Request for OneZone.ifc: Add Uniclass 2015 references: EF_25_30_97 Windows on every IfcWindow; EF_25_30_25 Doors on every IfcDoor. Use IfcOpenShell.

First a look at what the model holds.

```python
import ifcopenshell

model = ifcopenshell.open("OneZone.ifc")
print(model.schema)
print("classifications:", [c.Name for c in model.by_type("IfcClassification")])
for ifc_class in ("IfcDoor", "IfcRoof", "IfcStair", "IfcWall", "IfcWindow"):
    print(ifc_class, len(model.by_type(ifc_class)))
```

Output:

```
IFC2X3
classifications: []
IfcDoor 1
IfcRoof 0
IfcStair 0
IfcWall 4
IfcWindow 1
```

```python
import ifcopenshell
import ifcopenshell.api.classification

model = ifcopenshell.open("OneZone.ifc")

# IFC2X3 requires Source and Edition and has no link from the project to the system.
system = model.create_entity("IfcClassification", Source="NBS", Edition="2015", Name="Uniclass 2015")

codes = {
    "IfcWindow": ("EF_25_30_97", "Windows"),
    "IfcDoor": ("EF_25_30_25", "Doors"),
}
for ifc_class, (code, name) in codes.items():
    products = model.by_type(ifc_class)
    ifcopenshell.api.classification.add_reference(
        model, products=products, classification=system, identification=code, name=name
    )
    print(code, len(products))

model.write("OneZone_v2.ifc")
```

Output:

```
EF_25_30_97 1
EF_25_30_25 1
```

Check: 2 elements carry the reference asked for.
